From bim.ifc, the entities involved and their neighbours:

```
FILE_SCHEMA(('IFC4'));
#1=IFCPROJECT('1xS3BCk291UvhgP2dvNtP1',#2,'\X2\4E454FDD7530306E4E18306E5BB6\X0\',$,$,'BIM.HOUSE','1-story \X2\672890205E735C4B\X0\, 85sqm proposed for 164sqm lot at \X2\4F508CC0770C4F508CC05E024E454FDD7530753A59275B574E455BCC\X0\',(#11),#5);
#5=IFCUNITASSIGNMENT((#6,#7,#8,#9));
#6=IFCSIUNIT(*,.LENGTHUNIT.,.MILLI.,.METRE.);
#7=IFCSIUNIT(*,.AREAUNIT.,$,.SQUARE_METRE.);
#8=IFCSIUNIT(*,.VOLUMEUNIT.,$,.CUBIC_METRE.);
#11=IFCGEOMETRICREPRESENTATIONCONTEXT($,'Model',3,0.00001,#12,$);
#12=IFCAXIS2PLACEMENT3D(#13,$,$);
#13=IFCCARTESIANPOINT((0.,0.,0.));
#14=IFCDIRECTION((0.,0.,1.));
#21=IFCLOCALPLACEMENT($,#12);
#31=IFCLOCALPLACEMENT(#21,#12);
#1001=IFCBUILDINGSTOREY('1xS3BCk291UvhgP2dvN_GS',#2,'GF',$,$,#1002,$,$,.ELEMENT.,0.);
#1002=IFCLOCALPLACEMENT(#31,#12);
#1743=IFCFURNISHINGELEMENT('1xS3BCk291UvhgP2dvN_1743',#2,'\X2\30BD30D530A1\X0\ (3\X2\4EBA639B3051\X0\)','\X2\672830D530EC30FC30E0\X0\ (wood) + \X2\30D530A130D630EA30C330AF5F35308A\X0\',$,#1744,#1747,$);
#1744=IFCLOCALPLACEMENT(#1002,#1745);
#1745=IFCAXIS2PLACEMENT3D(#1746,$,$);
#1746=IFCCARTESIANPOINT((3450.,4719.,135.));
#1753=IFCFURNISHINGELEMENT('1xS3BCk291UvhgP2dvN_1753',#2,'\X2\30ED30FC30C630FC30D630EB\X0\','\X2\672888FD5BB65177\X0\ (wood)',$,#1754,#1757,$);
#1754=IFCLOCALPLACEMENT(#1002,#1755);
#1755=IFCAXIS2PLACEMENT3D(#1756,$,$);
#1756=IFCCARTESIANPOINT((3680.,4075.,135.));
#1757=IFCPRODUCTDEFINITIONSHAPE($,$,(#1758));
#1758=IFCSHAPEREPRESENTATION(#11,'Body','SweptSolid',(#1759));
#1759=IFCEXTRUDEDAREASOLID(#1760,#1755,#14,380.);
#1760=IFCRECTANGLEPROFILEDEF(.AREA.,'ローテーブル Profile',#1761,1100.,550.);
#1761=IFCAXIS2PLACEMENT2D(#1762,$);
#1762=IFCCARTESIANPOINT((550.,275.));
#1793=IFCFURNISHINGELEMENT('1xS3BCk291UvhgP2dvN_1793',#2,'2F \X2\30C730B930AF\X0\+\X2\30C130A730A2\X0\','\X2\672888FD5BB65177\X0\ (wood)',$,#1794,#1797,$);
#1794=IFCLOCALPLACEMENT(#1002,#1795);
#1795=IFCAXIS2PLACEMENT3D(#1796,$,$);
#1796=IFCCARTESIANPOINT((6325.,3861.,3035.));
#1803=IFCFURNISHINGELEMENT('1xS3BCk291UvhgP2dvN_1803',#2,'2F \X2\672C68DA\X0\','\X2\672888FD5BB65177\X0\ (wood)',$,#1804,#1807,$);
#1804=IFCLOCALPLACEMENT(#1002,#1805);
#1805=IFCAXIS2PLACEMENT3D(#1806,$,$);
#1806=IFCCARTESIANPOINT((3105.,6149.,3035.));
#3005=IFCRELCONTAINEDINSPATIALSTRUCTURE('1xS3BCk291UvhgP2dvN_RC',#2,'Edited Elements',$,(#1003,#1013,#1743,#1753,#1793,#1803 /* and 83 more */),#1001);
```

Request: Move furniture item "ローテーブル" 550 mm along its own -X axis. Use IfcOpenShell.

```python
import ifcopenshell
import ifcopenshell.api.geometry
import ifcopenshell.util.placement
import ifcopenshell.util.unit

model = ifcopenshell.open("bim.ifc")
unit_scale = ifcopenshell.util.unit.calculate_unit_scale(model)

item = model.by_guid("1xS3BCk291UvhgP2dvN_1753")
matrix = ifcopenshell.util.placement.get_local_placement(item.ObjectPlacement)
matrix[:3, 3] -= matrix[:3, 0] * 0.55 / unit_scale
ifcopenshell.api.geometry.edit_object_placement(model, product=item, matrix=matrix, is_si=False)

print(ifcopenshell.util.placement.get_local_placement(item.ObjectPlacement).round(3) + 0.0)

model.write("bim-out.ifc")
```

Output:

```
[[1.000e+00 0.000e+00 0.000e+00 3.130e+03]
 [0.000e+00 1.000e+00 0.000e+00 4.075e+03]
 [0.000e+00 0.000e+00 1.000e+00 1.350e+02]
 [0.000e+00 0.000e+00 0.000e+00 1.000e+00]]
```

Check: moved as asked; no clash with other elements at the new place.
